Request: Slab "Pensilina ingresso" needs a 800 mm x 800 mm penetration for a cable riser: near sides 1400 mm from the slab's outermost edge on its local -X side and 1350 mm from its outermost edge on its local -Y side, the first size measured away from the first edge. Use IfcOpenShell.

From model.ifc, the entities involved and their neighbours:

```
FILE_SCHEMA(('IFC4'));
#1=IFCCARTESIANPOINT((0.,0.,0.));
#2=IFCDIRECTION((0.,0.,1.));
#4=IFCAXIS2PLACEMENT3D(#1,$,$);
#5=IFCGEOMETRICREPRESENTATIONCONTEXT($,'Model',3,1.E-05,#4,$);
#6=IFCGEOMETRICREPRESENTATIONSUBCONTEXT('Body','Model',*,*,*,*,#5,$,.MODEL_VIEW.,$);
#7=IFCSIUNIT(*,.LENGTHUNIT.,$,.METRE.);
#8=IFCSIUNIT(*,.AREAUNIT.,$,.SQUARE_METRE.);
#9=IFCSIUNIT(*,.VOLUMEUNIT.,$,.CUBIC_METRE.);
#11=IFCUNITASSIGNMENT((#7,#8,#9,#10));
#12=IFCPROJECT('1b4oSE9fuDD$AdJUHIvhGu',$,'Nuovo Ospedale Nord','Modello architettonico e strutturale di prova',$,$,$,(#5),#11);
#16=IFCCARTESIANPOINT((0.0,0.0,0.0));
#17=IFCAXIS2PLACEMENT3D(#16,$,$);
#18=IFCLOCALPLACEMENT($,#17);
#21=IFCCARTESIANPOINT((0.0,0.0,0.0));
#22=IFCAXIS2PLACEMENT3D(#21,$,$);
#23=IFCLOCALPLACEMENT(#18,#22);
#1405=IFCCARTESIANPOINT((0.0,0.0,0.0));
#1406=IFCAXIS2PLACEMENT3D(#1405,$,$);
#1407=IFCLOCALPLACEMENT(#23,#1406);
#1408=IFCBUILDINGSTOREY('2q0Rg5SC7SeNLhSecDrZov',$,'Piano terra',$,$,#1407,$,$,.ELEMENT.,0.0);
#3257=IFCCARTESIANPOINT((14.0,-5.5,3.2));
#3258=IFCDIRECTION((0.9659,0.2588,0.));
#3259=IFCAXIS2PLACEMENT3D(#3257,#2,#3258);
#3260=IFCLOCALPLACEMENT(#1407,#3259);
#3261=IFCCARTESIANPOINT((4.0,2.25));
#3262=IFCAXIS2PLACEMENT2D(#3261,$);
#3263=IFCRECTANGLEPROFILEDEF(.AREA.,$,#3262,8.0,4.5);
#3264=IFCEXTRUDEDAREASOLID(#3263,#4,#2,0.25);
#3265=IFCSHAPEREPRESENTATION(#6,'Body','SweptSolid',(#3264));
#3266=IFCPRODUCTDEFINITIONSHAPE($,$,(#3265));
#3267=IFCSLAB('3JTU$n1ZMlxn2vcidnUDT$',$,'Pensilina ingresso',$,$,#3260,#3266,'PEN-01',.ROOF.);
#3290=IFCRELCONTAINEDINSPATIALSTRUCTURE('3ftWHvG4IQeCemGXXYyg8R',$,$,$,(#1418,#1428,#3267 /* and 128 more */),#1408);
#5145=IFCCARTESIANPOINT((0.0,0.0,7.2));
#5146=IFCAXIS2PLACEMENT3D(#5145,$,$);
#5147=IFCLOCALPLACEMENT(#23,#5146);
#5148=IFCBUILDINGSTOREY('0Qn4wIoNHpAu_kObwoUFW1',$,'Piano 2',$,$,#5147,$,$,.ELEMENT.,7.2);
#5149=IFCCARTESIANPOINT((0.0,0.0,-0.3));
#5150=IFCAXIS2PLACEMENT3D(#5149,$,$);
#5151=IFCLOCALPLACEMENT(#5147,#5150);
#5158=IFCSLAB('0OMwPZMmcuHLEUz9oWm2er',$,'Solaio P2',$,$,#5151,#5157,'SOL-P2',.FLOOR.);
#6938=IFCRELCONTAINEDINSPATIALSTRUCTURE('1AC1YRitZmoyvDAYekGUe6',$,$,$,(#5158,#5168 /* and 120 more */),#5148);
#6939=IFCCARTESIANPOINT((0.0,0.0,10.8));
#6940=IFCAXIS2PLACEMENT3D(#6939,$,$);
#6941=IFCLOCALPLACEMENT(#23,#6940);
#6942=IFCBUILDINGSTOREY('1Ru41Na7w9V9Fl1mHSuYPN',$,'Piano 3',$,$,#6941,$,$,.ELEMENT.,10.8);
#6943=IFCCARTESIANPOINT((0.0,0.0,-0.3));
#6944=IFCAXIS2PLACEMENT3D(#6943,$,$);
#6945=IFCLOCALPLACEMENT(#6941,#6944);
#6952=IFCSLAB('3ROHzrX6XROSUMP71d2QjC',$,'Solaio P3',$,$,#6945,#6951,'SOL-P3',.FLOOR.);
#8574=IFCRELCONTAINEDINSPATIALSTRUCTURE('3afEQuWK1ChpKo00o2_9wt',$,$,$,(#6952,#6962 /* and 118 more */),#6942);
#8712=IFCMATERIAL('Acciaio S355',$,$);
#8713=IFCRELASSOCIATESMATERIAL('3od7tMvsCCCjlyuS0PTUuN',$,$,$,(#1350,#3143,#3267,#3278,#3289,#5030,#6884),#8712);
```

```python
import numpy as np
import ifcopenshell
import ifcopenshell.api.feature
import ifcopenshell.api.geometry
import ifcopenshell.api.root
import ifcopenshell.geom
import ifcopenshell.util.placement
import ifcopenshell.util.representation
import ifcopenshell.util.shape
import ifcopenshell.util.unit

model = ifcopenshell.open("model.ifc")
unit_scale = ifcopenshell.util.unit.calculate_unit_scale(model)
settings = ifcopenshell.geom.settings()


def volume(element):
    """Net volume in cubic metres, openings subtracted."""
    shape = ifcopenshell.geom.create_shape(settings, element)
    return ifcopenshell.util.shape.get_volume(shape.geometry)


slab = model.by_id(3267)
before = volume(slab)

# Extent in the slab's own axes, in metres. The edges named are its -X and -Y sides.
slab_shape = ifcopenshell.geom.create_shape(settings, slab)
vertices = ifcopenshell.util.shape.get_vertices(slab_shape.geometry)
x_min, y_min, bottom = vertices.min(axis=0)
top = vertices[:, 2].max()

opening = ifcopenshell.api.root.create_entity(model, ifc_class="IfcOpeningElement", name="Cable riser opening", predefined_type="OPENING")
context = ifcopenshell.util.representation.get_context(model, "Model", "Body", "MODEL_VIEW")
width, depth = 0.8, 0.8
outline = [(0.0, 0.0), (width, 0.0), (width, depth), (0.0, depth), (0.0, 0.0)]
# Overshoot both faces by 50 mm so the cut is clean.
shape = ifcopenshell.api.geometry.add_slab_representation(
    model, context=context, depth=top - bottom + 0.1, polyline=outline
)
ifcopenshell.api.geometry.assign_representation(model, product=opening, representation=shape)

matrix = ifcopenshell.util.placement.get_local_placement(slab.ObjectPlacement)
matrix[:, 3] = matrix @ np.append(np.array([x_min + 1.4, y_min + 1.35, bottom - 0.05]) / unit_scale, 1.0)
ifcopenshell.api.geometry.edit_object_placement(model, product=opening, matrix=matrix, is_si=False)
ifcopenshell.api.feature.add_feature(model, feature=opening, element=slab)

after = volume(slab)

print(f"slab volume {before:.3f} -> {after:.3f} m3")

model.write("model-out.ifc")
```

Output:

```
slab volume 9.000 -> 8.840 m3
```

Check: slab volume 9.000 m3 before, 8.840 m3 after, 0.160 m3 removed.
